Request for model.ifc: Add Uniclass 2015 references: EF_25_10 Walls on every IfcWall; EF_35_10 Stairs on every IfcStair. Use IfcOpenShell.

First a look at what the model holds.

```python
import ifcopenshell

model = ifcopenshell.open("model.ifc")
print(model.schema)
print("classifications:", [c.Name for c in model.by_type("IfcClassification")])
for ifc_class in ("IfcDoor", "IfcRoof", "IfcStair", "IfcWall", "IfcWindow"):
    print(ifc_class, len(model.by_type(ifc_class)))
```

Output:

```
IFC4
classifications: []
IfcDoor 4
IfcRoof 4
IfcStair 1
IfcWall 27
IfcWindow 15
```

```python
import ifcopenshell
import ifcopenshell.api.classification

model = ifcopenshell.open("model.ifc")

system = ifcopenshell.api.classification.add_classification(model, classification="Uniclass 2015")

codes = {
    "IfcWall": ("EF_25_10", "Walls"),
    "IfcStair": ("EF_35_10", "Stairs"),
}
for ifc_class, (code, name) in codes.items():
    products = model.by_type(ifc_class)
    ifcopenshell.api.classification.add_reference(
        model, products=products, classification=system, identification=code, name=name
    )
    print(code, len(products))

model.write("model_edited.ifc")
```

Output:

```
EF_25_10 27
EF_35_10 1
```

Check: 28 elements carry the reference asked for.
